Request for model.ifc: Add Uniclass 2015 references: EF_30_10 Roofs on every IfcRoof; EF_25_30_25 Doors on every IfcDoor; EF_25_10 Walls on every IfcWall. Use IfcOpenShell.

First a look at what the model holds.

```python
import ifcopenshell

model = ifcopenshell.open("model.ifc")
print(model.schema)
print("classifications:", [c.Name for c in model.by_type("IfcClassification")])
for ifc_class in ("IfcDoor", "IfcRoof", "IfcStair", "IfcWall", "IfcWindow"):
    print(ifc_class, len(model.by_type(ifc_class)))
```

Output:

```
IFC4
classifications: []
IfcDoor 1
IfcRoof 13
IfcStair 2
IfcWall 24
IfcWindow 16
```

```python
import ifcopenshell
import ifcopenshell.api.classification

model = ifcopenshell.open("model.ifc")

system = ifcopenshell.api.classification.add_classification(model, classification="Uniclass 2015")

codes = {
    "IfcRoof": ("EF_30_10", "Roofs"),
    "IfcDoor": ("EF_25_30_25", "Doors"),
    "IfcWall": ("EF_25_10", "Walls"),
}
for ifc_class, (code, name) in codes.items():
    products = model.by_type(ifc_class)
    ifcopenshell.api.classification.add_reference(
        model, products=products, classification=system, identification=code, name=name
    )
    print(code, len(products))

model.write("model_v2.ifc")
```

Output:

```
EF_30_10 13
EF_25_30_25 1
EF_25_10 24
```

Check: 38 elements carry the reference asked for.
